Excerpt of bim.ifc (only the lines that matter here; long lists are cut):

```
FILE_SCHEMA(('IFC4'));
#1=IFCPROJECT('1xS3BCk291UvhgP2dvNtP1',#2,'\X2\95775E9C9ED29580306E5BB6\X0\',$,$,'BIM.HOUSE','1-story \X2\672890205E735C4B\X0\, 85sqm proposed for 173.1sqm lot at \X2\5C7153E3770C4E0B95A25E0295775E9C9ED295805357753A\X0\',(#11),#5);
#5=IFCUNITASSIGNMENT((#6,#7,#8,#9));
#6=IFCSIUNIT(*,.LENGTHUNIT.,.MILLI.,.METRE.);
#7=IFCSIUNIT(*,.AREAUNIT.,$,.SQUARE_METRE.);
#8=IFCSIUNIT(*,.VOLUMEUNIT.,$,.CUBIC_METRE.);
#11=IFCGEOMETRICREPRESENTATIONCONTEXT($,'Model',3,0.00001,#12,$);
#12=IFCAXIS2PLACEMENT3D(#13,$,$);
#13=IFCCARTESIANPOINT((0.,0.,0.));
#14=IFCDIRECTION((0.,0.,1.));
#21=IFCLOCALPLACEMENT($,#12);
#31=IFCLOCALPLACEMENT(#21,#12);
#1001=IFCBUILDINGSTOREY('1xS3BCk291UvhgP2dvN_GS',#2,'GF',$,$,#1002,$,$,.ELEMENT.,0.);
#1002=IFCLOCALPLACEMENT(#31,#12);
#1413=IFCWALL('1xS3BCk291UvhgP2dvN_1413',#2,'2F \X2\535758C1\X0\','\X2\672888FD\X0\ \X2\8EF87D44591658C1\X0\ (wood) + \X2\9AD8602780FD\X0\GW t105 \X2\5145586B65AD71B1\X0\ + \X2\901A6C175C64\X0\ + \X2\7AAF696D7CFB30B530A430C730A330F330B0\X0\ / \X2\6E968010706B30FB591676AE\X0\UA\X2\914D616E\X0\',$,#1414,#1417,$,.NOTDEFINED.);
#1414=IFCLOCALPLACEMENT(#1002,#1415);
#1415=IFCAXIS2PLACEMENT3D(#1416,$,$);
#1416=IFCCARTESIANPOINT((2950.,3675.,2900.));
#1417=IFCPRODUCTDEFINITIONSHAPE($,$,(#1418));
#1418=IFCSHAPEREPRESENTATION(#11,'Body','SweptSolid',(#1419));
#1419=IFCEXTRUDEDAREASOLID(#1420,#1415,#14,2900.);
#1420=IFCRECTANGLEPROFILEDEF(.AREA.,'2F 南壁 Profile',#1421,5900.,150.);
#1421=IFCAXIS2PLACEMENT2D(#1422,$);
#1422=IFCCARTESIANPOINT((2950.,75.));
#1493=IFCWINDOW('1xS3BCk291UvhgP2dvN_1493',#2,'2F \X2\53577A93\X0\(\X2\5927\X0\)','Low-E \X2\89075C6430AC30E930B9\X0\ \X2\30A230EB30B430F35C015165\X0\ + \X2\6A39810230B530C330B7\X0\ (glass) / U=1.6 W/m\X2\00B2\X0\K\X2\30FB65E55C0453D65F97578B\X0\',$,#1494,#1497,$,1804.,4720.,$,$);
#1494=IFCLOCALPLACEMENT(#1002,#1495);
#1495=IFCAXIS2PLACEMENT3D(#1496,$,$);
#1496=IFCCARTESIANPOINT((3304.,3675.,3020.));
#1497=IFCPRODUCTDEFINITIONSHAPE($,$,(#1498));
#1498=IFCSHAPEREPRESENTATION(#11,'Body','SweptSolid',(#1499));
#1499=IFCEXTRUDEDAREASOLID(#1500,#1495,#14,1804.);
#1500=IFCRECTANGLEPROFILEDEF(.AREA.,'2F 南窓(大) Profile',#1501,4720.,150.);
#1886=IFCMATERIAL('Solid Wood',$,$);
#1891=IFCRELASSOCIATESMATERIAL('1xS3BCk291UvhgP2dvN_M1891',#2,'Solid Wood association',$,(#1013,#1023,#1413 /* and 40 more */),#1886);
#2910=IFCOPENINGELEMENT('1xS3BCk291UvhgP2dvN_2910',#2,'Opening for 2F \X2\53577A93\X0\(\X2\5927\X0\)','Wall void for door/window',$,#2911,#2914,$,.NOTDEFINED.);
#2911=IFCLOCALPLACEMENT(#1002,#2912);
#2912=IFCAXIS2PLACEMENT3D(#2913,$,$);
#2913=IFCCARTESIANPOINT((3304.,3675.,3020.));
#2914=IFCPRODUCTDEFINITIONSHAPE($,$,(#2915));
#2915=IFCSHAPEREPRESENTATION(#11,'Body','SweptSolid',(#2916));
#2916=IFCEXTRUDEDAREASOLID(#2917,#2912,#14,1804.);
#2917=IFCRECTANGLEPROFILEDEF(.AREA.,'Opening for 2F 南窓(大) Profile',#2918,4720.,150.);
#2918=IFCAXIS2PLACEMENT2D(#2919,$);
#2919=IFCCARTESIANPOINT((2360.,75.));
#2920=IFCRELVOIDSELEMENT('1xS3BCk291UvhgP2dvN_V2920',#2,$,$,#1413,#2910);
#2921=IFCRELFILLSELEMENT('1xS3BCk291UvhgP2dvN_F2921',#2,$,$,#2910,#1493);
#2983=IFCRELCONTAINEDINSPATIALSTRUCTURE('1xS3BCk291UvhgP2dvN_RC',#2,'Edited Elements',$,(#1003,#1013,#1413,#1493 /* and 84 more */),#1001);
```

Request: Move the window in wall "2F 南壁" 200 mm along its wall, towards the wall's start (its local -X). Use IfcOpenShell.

```python
import ifcopenshell
import ifcopenshell.api.geometry
import ifcopenshell.util.placement
import ifcopenshell.util.unit

model = ifcopenshell.open("bim.ifc")
unit_scale = ifcopenshell.util.unit.calculate_unit_scale(model)

window = model.by_guid("1xS3BCk291UvhgP2dvN_1493")
opening = window.FillsVoids[0].RelatingOpeningElement
wall = opening.VoidsElements[0].RelatingBuildingElement

wall_matrix = ifcopenshell.util.placement.get_local_placement(wall.ObjectPlacement)
shift = wall_matrix[:3, 0] * -0.2 / unit_scale
before = ifcopenshell.util.placement.get_local_placement(window.ObjectPlacement)[:3, 3].copy()

# The window is not placed relative to its opening, so move both.
for product in (opening, window):
    matrix = ifcopenshell.util.placement.get_local_placement(product.ObjectPlacement)
    matrix[:3, 3] += shift
    ifcopenshell.api.geometry.edit_object_placement(model, product=product, matrix=matrix, is_si=False)

after = ifcopenshell.util.placement.get_local_placement(window.ObjectPlacement)[:3, 3]
print("window moved by", (after - before).round(3) + 0.0)

model.write("bim_rev.ifc")
```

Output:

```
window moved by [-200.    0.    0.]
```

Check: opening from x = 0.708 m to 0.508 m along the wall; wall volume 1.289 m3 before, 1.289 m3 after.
